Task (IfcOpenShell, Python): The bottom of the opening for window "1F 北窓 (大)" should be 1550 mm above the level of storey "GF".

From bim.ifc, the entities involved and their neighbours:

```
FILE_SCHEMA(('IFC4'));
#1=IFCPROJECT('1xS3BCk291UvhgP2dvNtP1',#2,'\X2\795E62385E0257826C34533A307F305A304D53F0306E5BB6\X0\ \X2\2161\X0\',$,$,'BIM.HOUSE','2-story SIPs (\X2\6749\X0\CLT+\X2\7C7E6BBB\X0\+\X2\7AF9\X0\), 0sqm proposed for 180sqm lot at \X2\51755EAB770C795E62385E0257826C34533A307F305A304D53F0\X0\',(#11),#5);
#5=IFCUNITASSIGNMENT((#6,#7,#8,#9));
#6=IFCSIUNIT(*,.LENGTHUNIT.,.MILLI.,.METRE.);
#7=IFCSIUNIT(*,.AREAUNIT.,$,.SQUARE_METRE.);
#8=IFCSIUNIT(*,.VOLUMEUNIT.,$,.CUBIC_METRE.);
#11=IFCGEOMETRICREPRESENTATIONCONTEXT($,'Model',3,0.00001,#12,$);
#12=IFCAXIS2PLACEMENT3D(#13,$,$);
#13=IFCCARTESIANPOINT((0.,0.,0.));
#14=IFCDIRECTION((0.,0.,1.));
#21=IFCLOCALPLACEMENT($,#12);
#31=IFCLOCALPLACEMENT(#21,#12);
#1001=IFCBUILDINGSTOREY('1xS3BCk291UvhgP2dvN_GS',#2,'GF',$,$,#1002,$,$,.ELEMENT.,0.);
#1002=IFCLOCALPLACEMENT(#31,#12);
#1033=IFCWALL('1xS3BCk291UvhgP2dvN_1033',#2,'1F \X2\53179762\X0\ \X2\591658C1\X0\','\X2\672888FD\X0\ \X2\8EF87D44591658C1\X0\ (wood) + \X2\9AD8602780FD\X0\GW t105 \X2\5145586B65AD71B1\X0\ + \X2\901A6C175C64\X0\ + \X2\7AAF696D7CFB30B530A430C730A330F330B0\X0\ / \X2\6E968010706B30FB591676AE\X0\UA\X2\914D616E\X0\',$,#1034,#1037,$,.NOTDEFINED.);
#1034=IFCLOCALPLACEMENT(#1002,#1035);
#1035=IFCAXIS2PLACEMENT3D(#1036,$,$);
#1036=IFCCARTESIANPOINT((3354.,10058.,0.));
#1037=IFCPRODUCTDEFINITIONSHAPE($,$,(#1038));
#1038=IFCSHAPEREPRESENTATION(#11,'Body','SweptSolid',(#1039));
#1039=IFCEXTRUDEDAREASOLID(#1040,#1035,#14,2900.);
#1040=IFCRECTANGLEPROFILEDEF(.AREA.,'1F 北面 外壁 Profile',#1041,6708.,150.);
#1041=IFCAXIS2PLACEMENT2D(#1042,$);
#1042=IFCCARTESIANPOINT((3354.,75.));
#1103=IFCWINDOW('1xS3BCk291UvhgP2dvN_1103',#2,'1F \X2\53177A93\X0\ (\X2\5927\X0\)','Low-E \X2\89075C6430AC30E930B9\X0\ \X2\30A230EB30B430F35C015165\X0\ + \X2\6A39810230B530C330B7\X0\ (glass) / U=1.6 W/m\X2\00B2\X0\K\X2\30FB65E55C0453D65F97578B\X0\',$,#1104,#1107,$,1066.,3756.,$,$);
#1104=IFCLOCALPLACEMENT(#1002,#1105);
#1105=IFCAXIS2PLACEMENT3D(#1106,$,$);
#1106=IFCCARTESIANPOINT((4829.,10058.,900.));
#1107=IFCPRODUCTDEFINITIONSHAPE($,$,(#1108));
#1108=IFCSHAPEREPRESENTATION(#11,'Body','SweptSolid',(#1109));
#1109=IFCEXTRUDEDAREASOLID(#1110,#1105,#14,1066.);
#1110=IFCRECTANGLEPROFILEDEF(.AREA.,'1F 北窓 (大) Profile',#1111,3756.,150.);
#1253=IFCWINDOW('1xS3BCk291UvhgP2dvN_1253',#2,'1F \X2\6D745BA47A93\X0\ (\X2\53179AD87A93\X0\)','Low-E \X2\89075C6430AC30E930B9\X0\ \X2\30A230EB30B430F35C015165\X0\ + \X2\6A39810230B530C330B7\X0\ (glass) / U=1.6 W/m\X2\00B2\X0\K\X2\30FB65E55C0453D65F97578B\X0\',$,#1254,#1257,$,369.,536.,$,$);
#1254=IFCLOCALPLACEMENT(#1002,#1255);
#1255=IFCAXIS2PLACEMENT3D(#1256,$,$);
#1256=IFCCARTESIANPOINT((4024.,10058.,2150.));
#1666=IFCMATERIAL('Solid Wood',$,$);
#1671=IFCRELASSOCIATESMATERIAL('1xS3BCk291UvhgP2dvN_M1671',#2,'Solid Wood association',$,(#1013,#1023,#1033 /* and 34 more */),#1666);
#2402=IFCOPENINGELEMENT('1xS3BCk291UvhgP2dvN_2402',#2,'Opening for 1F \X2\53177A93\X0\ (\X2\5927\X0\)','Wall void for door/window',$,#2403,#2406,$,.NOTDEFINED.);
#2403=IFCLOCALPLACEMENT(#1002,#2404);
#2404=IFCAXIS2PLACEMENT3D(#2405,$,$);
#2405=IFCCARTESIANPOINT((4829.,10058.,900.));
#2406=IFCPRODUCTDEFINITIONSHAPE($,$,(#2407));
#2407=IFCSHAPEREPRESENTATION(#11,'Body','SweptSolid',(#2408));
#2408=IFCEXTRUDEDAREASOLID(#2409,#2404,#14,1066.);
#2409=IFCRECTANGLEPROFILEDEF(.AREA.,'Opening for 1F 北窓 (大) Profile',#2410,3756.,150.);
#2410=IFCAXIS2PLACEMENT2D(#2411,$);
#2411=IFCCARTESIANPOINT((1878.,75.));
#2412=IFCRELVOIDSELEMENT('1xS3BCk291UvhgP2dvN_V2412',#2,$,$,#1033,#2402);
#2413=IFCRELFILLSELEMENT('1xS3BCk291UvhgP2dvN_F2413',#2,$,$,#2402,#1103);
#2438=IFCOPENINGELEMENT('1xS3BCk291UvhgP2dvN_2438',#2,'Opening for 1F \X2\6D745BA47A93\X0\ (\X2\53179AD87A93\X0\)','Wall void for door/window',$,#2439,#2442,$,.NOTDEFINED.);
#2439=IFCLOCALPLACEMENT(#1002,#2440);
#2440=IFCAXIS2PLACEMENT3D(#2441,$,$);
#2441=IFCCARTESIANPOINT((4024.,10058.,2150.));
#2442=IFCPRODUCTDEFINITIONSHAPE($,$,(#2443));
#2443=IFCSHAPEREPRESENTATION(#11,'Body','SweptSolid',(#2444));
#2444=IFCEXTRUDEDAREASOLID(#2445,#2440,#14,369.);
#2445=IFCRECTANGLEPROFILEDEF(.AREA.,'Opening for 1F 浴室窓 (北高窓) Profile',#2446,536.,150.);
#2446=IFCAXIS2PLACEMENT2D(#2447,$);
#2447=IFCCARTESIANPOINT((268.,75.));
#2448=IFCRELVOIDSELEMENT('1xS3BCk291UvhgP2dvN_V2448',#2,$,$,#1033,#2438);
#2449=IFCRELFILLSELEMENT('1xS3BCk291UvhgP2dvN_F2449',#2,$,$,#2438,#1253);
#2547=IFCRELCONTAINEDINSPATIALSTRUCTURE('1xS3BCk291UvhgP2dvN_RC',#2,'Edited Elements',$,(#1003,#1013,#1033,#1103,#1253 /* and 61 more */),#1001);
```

```python
import numpy as np
import ifcopenshell
import ifcopenshell.api.geometry
import ifcopenshell.geom
import ifcopenshell.util.element
import ifcopenshell.util.placement
import ifcopenshell.util.shape
import ifcopenshell.util.unit

model = ifcopenshell.open("bim.ifc")
unit_scale = ifcopenshell.util.unit.calculate_unit_scale(model)

window = model.by_id(1103)
opening = window.FillsVoids[0].RelatingOpeningElement
storey = ifcopenshell.util.element.get_container(window, ifc_class="IfcBuildingStorey")
level = ifcopenshell.util.placement.get_local_placement(storey.ObjectPlacement)[2, 3]

# The opening's origin need not be at the sill, so measure its lowest point.
shape = ifcopenshell.geom.create_shape(ifcopenshell.geom.settings(), opening)
bottom = ifcopenshell.util.shape.get_shape_bottom_elevation(shape, shape.geometry) / unit_scale
dz = level + 1550.0 - bottom

shift = np.array([0.0, 0.0, dz])
# The window is not placed relative to its opening, so move both.
for product in (opening, window):
    matrix = ifcopenshell.util.placement.get_local_placement(product.ObjectPlacement)
    matrix[:3, 3] += shift
    ifcopenshell.api.geometry.edit_object_placement(model, product=product, matrix=matrix, is_si=False)

print(f"moved by {dz * unit_scale:+.3f} m")

model.write("bim_v2.ifc")
```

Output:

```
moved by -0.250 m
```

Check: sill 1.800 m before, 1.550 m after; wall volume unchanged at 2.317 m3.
